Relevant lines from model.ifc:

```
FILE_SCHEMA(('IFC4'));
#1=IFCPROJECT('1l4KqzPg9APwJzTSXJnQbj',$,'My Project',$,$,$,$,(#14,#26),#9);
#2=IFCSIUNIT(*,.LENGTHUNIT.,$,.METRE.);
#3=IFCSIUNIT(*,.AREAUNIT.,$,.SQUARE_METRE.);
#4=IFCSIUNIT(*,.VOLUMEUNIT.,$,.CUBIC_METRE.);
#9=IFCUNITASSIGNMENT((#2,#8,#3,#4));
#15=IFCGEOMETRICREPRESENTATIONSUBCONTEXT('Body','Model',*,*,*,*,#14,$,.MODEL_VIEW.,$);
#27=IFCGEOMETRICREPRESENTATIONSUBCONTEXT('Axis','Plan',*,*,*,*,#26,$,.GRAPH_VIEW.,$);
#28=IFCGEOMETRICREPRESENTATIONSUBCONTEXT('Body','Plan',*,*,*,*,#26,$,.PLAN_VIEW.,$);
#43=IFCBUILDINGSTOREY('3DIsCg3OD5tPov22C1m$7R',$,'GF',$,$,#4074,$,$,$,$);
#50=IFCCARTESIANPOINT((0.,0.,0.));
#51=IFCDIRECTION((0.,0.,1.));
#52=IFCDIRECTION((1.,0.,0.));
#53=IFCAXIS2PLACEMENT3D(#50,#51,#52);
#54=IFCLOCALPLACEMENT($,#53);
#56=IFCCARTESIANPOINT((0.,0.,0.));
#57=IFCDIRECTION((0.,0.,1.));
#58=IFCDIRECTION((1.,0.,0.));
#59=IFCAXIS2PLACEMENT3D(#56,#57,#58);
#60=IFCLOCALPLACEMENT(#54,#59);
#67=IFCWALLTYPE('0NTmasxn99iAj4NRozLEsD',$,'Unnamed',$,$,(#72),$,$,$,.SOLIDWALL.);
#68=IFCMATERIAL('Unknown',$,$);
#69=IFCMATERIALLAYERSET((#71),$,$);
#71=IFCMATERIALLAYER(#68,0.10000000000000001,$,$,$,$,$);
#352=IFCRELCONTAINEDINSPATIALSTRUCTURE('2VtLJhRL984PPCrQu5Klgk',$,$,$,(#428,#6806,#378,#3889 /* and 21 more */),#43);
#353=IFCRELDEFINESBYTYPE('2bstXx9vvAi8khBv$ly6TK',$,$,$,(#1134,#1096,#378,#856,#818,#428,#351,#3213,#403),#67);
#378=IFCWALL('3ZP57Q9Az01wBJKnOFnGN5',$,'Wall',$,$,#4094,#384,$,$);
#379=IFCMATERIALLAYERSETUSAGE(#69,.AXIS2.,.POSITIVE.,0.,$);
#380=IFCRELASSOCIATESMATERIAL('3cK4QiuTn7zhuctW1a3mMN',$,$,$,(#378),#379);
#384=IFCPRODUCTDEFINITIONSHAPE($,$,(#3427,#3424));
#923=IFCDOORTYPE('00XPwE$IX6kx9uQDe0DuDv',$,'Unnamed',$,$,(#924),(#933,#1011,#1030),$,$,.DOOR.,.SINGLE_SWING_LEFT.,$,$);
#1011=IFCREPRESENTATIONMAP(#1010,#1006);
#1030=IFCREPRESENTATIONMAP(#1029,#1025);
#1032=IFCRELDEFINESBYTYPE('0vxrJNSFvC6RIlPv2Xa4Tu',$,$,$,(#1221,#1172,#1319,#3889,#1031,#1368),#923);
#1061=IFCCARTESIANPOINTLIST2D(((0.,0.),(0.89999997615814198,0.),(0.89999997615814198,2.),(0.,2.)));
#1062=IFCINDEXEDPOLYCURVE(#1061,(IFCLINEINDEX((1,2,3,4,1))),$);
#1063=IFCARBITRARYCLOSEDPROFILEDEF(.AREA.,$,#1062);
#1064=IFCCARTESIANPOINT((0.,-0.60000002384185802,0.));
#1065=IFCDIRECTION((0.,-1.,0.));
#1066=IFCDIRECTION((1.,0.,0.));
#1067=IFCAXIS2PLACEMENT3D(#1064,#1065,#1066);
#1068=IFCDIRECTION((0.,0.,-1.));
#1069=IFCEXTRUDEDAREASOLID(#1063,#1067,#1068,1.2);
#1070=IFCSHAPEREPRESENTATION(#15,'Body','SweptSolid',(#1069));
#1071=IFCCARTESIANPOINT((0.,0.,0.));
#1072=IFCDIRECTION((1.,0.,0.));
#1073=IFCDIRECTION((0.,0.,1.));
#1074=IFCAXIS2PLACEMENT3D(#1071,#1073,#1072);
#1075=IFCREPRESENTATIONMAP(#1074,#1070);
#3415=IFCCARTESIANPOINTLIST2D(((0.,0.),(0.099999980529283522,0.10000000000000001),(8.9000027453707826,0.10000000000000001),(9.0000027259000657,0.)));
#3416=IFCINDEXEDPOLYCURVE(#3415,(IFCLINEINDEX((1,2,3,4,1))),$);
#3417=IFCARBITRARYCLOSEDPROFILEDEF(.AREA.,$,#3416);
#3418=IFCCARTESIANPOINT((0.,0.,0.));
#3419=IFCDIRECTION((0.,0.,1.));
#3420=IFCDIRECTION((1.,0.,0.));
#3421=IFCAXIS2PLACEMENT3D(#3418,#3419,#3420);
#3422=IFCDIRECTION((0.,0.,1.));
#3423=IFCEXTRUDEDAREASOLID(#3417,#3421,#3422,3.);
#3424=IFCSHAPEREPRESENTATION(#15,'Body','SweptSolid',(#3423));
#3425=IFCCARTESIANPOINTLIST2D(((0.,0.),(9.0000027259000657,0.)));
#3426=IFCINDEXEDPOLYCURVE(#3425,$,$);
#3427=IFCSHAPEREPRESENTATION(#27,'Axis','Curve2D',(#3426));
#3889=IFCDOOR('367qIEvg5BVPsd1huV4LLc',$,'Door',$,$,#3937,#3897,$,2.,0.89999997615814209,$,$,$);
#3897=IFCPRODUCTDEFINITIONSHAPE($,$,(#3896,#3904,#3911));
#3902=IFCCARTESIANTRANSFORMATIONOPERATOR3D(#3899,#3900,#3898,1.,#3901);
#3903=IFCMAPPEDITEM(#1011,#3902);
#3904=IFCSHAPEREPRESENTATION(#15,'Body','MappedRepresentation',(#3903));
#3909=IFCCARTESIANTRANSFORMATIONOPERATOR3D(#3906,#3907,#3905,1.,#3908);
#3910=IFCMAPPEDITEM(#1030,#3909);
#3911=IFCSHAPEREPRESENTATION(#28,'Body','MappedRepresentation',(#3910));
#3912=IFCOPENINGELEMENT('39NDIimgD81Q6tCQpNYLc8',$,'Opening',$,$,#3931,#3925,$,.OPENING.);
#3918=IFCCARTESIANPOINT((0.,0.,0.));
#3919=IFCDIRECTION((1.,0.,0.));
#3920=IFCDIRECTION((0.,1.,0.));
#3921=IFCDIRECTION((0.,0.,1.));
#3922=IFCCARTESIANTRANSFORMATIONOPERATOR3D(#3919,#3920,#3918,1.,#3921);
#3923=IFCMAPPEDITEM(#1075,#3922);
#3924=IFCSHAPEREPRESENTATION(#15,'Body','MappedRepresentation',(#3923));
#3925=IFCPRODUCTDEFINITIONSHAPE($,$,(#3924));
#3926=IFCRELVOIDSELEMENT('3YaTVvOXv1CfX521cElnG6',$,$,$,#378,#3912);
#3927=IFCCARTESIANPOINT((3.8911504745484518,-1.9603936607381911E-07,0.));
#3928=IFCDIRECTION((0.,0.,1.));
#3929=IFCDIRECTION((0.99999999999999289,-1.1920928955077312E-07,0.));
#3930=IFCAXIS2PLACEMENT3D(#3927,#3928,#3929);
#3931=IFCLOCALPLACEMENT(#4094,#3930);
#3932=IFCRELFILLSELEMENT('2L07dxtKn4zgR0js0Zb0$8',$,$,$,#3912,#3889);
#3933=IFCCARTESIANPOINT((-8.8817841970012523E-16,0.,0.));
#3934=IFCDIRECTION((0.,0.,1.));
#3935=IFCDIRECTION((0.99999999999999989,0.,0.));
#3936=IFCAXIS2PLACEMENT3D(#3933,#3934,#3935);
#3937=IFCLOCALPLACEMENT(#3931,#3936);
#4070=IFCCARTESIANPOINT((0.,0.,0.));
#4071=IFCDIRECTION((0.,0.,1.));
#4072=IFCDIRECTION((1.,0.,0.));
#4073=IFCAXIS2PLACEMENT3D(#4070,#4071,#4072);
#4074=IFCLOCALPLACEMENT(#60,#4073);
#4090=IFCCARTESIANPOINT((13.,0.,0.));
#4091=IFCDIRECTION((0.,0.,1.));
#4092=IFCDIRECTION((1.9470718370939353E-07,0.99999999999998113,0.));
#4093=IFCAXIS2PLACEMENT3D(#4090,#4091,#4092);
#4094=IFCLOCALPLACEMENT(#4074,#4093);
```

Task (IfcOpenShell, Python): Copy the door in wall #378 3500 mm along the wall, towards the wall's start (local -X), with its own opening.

```python
import ifcopenshell
import ifcopenshell.api.feature
import ifcopenshell.api.geometry
import ifcopenshell.api.root
import ifcopenshell.geom
import ifcopenshell.util.element
import ifcopenshell.util.placement
import ifcopenshell.util.shape
import ifcopenshell.util.unit

model = ifcopenshell.open("model.ifc")
unit_scale = ifcopenshell.util.unit.calculate_unit_scale(model)
settings = ifcopenshell.geom.settings()


def volume(element):
    """Net volume in cubic metres, openings subtracted."""
    shape = ifcopenshell.geom.create_shape(settings, element)
    return ifcopenshell.util.shape.get_volume(shape.geometry)


door = model.by_guid("367qIEvg5BVPsd1huV4LLc")
opening = door.FillsVoids[0].RelatingOpeningElement
wall = opening.VoidsElements[0].RelatingBuildingElement
before = volume(wall)
shift = ifcopenshell.util.placement.get_local_placement(wall.ObjectPlacement)[:3, 0] * -3.5 / unit_scale

# copy_class copies the void relationship, type, container and properties, but no geometry.
new_opening = ifcopenshell.api.root.copy_class(model, product=opening)
new_opening.Representation = ifcopenshell.util.element.copy_deep(
    model, opening.Representation, exclude=["IfcGeometricRepresentationContext", "IfcRepresentationMap"]
)
new_door = ifcopenshell.api.root.copy_class(model, product=door)
new_door.Representation = ifcopenshell.util.element.copy_deep(
    model, door.Representation, exclude=["IfcGeometricRepresentationContext", "IfcRepresentationMap"]
)
ifcopenshell.api.feature.add_filling(model, opening=new_opening, element=new_door)

for old, new in ((opening, new_opening), (door, new_door)):
    matrix = ifcopenshell.util.placement.get_local_placement(old.ObjectPlacement)
    matrix[:3, 3] += shift
    ifcopenshell.api.geometry.edit_object_placement(model, product=new, matrix=matrix, is_si=False)

after = volume(wall)

print(f"wall volume {before:.3f} -> {after:.3f} m3")

model.write("model_v2.ifc")
```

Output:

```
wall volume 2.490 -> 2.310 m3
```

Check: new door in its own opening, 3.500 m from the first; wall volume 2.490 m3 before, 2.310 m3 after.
